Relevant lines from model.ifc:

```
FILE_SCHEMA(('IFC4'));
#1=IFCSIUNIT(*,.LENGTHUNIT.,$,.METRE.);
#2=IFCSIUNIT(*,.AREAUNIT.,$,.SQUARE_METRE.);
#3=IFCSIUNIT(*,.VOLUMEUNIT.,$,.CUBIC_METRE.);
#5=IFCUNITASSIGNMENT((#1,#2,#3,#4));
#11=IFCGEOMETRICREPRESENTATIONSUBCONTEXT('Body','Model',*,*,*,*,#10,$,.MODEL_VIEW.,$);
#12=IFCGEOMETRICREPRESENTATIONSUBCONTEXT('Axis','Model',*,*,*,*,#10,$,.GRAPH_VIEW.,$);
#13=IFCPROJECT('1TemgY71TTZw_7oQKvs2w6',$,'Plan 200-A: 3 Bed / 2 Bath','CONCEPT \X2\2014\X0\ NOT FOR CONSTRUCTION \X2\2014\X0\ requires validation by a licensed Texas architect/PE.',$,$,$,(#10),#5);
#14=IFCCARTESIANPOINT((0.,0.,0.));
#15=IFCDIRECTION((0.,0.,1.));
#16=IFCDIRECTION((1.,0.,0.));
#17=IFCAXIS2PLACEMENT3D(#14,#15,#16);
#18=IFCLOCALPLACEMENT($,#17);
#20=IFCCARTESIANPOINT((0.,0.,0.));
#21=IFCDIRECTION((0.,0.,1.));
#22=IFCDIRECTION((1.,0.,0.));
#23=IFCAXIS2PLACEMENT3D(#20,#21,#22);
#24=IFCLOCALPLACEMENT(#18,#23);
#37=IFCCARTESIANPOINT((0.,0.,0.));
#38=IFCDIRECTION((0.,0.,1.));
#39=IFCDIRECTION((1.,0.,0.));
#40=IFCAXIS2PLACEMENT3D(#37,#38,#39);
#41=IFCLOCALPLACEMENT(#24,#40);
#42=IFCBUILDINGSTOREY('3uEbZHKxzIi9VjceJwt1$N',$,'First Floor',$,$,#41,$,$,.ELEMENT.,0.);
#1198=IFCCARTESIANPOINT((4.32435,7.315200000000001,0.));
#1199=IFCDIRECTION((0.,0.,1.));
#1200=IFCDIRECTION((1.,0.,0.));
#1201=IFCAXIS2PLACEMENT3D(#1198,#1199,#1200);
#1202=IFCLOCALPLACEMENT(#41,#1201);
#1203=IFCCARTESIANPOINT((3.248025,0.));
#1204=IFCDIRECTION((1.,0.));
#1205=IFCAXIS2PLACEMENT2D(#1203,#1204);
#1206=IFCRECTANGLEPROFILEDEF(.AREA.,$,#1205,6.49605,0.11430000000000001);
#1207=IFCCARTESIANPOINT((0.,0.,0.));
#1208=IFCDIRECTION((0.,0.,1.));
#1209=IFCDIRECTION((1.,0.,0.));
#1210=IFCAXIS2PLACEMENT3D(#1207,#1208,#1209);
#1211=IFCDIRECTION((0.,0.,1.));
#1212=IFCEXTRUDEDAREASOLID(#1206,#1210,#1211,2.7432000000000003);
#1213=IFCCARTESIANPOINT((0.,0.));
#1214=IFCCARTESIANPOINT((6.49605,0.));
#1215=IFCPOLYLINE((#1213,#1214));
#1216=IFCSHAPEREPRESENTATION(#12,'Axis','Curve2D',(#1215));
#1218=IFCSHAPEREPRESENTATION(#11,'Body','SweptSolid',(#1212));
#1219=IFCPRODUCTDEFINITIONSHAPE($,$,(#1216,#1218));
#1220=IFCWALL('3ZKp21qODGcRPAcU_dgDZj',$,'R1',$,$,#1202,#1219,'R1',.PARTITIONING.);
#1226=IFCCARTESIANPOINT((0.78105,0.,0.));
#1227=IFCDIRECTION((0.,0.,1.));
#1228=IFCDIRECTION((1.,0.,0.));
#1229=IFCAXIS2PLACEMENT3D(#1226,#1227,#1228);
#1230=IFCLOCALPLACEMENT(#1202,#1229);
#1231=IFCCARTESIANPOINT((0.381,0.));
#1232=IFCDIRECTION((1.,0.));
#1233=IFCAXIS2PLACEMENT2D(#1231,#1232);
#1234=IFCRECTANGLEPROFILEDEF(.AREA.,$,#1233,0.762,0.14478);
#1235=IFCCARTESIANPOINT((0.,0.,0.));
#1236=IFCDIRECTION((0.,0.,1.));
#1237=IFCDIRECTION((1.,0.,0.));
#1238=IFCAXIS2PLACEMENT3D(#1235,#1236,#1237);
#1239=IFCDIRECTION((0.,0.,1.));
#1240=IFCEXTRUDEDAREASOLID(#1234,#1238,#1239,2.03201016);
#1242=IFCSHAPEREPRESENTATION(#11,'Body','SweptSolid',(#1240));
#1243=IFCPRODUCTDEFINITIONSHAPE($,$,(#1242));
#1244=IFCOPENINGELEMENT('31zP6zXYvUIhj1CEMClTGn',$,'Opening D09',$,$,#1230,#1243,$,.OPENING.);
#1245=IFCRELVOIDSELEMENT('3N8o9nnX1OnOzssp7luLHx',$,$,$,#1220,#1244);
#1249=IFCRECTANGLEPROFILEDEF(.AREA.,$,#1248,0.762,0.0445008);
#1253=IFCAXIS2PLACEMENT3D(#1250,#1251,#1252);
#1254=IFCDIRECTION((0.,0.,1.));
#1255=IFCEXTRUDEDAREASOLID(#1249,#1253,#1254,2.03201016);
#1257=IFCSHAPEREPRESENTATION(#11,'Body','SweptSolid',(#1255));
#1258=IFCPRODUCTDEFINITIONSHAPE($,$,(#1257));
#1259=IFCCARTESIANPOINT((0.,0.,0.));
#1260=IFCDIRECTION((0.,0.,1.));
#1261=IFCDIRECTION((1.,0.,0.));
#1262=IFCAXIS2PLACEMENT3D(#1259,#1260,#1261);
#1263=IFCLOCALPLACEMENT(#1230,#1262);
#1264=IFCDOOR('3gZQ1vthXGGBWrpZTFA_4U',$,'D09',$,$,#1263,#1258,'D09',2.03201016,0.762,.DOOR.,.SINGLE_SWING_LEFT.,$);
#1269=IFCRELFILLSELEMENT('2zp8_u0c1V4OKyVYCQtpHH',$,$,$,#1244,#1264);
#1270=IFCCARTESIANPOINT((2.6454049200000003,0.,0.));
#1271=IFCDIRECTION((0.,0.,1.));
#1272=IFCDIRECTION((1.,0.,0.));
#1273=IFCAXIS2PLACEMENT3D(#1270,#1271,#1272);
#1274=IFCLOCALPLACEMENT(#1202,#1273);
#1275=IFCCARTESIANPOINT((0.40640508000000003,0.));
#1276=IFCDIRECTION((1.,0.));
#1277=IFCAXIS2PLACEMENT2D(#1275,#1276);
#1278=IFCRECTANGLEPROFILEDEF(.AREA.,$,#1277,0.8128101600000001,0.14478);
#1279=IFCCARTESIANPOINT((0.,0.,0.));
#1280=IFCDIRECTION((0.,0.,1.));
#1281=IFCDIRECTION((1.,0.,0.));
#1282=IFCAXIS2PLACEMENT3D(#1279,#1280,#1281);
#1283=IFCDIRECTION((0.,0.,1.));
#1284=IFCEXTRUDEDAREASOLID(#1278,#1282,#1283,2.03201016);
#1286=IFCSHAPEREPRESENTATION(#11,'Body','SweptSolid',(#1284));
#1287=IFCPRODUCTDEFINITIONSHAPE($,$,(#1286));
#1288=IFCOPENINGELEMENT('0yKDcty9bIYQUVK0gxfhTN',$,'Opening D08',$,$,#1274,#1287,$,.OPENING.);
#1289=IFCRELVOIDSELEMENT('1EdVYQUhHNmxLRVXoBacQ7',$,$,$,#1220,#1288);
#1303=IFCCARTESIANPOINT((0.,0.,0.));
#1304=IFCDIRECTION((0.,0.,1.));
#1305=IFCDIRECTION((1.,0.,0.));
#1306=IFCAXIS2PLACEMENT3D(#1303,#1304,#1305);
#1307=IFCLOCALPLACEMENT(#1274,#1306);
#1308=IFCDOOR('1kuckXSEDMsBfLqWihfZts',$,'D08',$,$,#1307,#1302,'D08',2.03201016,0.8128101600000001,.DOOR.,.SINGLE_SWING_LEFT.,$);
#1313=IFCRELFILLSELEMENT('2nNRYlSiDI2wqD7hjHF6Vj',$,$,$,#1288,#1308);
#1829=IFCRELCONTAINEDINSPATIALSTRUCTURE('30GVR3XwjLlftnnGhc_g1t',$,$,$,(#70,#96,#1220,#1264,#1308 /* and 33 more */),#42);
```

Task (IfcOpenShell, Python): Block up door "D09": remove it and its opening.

```python
import ifcopenshell
import ifcopenshell.api.feature
import ifcopenshell.api.root
import ifcopenshell.geom
import ifcopenshell.util.shape

model = ifcopenshell.open("model.ifc")
settings = ifcopenshell.geom.settings()


def volume(element):
    """Net volume in cubic metres, openings subtracted."""
    shape = ifcopenshell.geom.create_shape(settings, element)
    return ifcopenshell.util.shape.get_volume(shape.geometry)


door = model.by_guid("3gZQ1vthXGGBWrpZTFA_4U")
opening = door.FillsVoids[0].RelatingOpeningElement
wall = opening.VoidsElements[0].RelatingBuildingElement
before = volume(wall)

ifcopenshell.api.root.remove_product(model, product=door)
ifcopenshell.api.feature.remove_feature(model, feature=opening)

after = volume(wall)

print(f"wall volume {before:.3f} -> {after:.3f} m3")

model.write("model_edited.ifc")
```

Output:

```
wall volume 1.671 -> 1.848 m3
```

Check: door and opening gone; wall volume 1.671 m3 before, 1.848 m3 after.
